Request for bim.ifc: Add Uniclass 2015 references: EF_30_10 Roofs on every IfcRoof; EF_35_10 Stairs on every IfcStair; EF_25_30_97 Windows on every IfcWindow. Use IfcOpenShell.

First a look at what the model holds.

```python
import ifcopenshell

model = ifcopenshell.open("bim.ifc")
print(model.schema)
print("classifications:", [c.Name for c in model.by_type("IfcClassification")])
for ifc_class in ("IfcDoor", "IfcRoof", "IfcStair", "IfcWall", "IfcWindow"):
    print(ifc_class, len(model.by_type(ifc_class)))
```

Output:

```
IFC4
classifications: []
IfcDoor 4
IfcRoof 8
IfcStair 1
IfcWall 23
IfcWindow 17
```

```python
import ifcopenshell
import ifcopenshell.api.classification

model = ifcopenshell.open("bim.ifc")

system = ifcopenshell.api.classification.add_classification(model, classification="Uniclass 2015")

codes = {
    "IfcRoof": ("EF_30_10", "Roofs"),
    "IfcStair": ("EF_35_10", "Stairs"),
    "IfcWindow": ("EF_25_30_97", "Windows"),
}
for ifc_class, (code, name) in codes.items():
    products = model.by_type(ifc_class)
    ifcopenshell.api.classification.add_reference(
        model, products=products, classification=system, identification=code, name=name
    )
    print(code, len(products))

model.write("bim_updated.ifc")
```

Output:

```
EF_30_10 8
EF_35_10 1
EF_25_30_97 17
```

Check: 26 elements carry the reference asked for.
